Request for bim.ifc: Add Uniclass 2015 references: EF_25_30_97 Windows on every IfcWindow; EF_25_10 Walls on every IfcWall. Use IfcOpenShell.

First a look at what the model holds.

```python
import ifcopenshell

model = ifcopenshell.open("bim.ifc")
print(model.schema)
print("classifications:", [c.Name for c in model.by_type("IfcClassification")])
for ifc_class in ("IfcDoor", "IfcRoof", "IfcStair", "IfcWall", "IfcWindow"):
    print(ifc_class, len(model.by_type(ifc_class)))
```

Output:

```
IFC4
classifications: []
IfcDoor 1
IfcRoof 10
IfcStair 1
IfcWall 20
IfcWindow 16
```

```python
import ifcopenshell
import ifcopenshell.api.classification

model = ifcopenshell.open("bim.ifc")

system = ifcopenshell.api.classification.add_classification(model, classification="Uniclass 2015")

codes = {
    "IfcWindow": ("EF_25_30_97", "Windows"),
    "IfcWall": ("EF_25_10", "Walls"),
}
for ifc_class, (code, name) in codes.items():
    products = model.by_type(ifc_class)
    ifcopenshell.api.classification.add_reference(
        model, products=products, classification=system, identification=code, name=name
    )
    print(code, len(products))

model.write("bim_edited.ifc")
```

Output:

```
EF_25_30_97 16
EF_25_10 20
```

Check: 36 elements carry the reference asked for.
